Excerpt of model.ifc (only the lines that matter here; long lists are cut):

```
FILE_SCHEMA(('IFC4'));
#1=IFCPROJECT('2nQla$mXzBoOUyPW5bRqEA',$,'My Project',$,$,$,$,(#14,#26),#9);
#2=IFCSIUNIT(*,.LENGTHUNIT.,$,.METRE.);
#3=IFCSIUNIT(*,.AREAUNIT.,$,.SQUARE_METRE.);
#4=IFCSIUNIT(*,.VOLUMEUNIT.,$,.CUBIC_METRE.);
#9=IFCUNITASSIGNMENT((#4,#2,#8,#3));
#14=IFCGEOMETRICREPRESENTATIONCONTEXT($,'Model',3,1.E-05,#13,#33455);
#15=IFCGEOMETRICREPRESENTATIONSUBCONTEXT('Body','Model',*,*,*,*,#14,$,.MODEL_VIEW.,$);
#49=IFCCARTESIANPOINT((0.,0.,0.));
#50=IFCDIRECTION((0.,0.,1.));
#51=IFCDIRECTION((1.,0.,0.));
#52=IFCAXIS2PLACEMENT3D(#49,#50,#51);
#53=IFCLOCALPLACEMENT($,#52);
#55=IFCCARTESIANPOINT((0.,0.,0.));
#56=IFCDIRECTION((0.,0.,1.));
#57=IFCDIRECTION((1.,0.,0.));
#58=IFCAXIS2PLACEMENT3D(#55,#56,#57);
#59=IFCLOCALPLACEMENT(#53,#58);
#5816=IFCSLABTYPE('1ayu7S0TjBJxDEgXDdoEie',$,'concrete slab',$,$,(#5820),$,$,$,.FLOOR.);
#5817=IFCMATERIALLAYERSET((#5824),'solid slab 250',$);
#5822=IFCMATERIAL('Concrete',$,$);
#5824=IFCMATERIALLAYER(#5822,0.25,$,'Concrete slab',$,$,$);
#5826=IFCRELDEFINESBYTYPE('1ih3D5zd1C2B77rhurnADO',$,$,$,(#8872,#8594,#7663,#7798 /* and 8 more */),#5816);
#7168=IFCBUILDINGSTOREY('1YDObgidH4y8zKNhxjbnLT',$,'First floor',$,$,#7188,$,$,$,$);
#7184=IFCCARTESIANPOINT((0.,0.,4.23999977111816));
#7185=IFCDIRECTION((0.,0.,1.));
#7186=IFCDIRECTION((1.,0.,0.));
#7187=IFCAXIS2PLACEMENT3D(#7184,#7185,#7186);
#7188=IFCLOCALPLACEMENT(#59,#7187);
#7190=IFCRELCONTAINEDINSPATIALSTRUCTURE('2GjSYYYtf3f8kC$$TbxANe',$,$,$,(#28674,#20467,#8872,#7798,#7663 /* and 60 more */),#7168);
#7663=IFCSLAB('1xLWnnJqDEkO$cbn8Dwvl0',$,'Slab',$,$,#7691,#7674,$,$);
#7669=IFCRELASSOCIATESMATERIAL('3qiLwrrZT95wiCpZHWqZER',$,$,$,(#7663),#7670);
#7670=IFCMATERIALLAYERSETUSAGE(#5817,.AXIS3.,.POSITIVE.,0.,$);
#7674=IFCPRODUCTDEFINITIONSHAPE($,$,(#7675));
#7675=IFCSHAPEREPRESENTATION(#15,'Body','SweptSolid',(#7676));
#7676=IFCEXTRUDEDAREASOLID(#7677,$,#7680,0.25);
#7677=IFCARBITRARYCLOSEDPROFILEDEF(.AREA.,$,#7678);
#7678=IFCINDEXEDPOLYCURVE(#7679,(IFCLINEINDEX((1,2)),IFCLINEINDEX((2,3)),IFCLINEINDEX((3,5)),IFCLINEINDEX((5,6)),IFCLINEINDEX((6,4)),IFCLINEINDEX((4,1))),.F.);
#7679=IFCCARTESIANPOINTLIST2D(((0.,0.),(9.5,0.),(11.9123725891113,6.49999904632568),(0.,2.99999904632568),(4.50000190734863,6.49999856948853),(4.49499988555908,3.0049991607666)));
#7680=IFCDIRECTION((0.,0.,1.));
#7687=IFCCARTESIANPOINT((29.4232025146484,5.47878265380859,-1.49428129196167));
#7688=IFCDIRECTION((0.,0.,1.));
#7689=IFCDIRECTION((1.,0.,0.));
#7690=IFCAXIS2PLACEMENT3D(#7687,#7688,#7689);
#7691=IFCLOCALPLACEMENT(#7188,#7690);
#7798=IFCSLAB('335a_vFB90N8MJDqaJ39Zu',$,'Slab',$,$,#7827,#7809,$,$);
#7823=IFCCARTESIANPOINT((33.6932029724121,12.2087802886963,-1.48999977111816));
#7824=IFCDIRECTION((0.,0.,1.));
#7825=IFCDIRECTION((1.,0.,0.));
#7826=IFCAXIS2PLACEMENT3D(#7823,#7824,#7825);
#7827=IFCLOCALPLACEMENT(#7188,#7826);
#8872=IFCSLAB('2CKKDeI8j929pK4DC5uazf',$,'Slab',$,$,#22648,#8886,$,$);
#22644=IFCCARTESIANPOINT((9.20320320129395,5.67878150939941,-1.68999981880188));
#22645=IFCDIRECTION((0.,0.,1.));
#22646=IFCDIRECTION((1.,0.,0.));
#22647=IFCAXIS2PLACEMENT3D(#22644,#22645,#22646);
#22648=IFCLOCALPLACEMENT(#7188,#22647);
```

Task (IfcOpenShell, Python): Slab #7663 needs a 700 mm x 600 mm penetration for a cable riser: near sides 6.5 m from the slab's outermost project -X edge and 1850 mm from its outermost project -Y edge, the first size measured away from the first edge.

```python
import numpy as np
import ifcopenshell
import ifcopenshell.api.feature
import ifcopenshell.api.geometry
import ifcopenshell.api.root
import ifcopenshell.geom
import ifcopenshell.util.placement
import ifcopenshell.util.representation
import ifcopenshell.util.shape
import ifcopenshell.util.unit

model = ifcopenshell.open("model.ifc")
unit_scale = ifcopenshell.util.unit.calculate_unit_scale(model)
settings = ifcopenshell.geom.settings()


def volume(element):
    """Net volume in cubic metres, openings subtracted."""
    shape = ifcopenshell.geom.create_shape(settings, element)
    return ifcopenshell.util.shape.get_volume(shape.geometry)


slab = model.by_guid("1xLWnnJqDEkO$cbn8Dwvl0")
before = volume(slab)

# Extent in the slab's own axes, in metres. The edges named are its -X and -Y sides.
slab_shape = ifcopenshell.geom.create_shape(settings, slab)
vertices = ifcopenshell.util.shape.get_vertices(slab_shape.geometry)
x_min, y_min, bottom = vertices.min(axis=0)
top = vertices[:, 2].max()

opening = ifcopenshell.api.root.create_entity(model, ifc_class="IfcOpeningElement", name="Cable riser opening", predefined_type="OPENING")
context = ifcopenshell.util.representation.get_context(model, "Model", "Body", "MODEL_VIEW")
width, depth = 0.7, 0.6
outline = [(0.0, 0.0), (width, 0.0), (width, depth), (0.0, depth), (0.0, 0.0)]
# Overshoot both faces by 50 mm so the cut is clean.
shape = ifcopenshell.api.geometry.add_slab_representation(
    model, context=context, depth=top - bottom + 0.1, polyline=outline
)
ifcopenshell.api.geometry.assign_representation(model, product=opening, representation=shape)

matrix = ifcopenshell.util.placement.get_local_placement(slab.ObjectPlacement)
matrix[:, 3] = matrix @ np.append(np.array([x_min + 6.5, y_min + 1.85, bottom - 0.05]) / unit_scale, 1.0)
ifcopenshell.api.geometry.edit_object_placement(model, product=opening, matrix=matrix, is_si=False)
ifcopenshell.api.feature.add_feature(model, feature=opening, element=slab)

after = volume(slab)

print(f"slab volume {before:.3f} -> {after:.3f} m3")

model.write("model_updated.ifc")
```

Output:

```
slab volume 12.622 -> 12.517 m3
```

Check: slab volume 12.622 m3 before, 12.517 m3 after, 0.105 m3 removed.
